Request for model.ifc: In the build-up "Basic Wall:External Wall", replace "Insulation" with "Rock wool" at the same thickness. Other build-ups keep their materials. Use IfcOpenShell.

First a look at what the model holds.

```python
import ifcopenshell
import ifcopenshell.util.element

model = ifcopenshell.open("model.ifc")
print(model.schema)
for layer_set in model.by_type("IfcMaterialLayerSet"):
    if layer_set.LayerSetName == "Basic Wall:External Wall":
        for layer in layer_set.MaterialLayers:
            print(layer.id(), layer.Material and layer.Material.Name, layer.LayerThickness, sep=" | ")
        print(len(ifcopenshell.util.element.get_elements_by_material(model, layer_set)), "elements and types use it")
print(sorted(m.Name for m in model.by_type("IfcMaterial") if m.Name)[:60])
```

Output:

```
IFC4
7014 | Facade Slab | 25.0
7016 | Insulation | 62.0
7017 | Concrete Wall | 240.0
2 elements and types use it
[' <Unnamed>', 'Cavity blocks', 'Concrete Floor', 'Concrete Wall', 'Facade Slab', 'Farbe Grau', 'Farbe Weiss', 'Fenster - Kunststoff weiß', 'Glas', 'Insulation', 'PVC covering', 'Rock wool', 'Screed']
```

```python
import ifcopenshell
import ifcopenshell.api.material

model = ifcopenshell.open("model.ifc")

layer_set = next(s for s in model.by_type("IfcMaterialLayerSet") if s.LayerSetName == "Basic Wall:External Wall")
layer = next(l for l in layer_set.MaterialLayers if l.Material and l.Material.Name == "Insulation")
material = next(m for m in model.by_type("IfcMaterial") if m.Name == "Rock wool")

# Point this one layer at the other material; renaming the old one would change it everywhere.
ifcopenshell.api.material.edit_layer(model, layer=layer, attributes={}, material=material)

print([l.Material.Name if l.Material else None for l in layer_set.MaterialLayers])

model.write("model_rev.ifc")
```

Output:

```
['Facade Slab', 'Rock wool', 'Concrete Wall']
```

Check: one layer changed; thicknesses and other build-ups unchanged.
